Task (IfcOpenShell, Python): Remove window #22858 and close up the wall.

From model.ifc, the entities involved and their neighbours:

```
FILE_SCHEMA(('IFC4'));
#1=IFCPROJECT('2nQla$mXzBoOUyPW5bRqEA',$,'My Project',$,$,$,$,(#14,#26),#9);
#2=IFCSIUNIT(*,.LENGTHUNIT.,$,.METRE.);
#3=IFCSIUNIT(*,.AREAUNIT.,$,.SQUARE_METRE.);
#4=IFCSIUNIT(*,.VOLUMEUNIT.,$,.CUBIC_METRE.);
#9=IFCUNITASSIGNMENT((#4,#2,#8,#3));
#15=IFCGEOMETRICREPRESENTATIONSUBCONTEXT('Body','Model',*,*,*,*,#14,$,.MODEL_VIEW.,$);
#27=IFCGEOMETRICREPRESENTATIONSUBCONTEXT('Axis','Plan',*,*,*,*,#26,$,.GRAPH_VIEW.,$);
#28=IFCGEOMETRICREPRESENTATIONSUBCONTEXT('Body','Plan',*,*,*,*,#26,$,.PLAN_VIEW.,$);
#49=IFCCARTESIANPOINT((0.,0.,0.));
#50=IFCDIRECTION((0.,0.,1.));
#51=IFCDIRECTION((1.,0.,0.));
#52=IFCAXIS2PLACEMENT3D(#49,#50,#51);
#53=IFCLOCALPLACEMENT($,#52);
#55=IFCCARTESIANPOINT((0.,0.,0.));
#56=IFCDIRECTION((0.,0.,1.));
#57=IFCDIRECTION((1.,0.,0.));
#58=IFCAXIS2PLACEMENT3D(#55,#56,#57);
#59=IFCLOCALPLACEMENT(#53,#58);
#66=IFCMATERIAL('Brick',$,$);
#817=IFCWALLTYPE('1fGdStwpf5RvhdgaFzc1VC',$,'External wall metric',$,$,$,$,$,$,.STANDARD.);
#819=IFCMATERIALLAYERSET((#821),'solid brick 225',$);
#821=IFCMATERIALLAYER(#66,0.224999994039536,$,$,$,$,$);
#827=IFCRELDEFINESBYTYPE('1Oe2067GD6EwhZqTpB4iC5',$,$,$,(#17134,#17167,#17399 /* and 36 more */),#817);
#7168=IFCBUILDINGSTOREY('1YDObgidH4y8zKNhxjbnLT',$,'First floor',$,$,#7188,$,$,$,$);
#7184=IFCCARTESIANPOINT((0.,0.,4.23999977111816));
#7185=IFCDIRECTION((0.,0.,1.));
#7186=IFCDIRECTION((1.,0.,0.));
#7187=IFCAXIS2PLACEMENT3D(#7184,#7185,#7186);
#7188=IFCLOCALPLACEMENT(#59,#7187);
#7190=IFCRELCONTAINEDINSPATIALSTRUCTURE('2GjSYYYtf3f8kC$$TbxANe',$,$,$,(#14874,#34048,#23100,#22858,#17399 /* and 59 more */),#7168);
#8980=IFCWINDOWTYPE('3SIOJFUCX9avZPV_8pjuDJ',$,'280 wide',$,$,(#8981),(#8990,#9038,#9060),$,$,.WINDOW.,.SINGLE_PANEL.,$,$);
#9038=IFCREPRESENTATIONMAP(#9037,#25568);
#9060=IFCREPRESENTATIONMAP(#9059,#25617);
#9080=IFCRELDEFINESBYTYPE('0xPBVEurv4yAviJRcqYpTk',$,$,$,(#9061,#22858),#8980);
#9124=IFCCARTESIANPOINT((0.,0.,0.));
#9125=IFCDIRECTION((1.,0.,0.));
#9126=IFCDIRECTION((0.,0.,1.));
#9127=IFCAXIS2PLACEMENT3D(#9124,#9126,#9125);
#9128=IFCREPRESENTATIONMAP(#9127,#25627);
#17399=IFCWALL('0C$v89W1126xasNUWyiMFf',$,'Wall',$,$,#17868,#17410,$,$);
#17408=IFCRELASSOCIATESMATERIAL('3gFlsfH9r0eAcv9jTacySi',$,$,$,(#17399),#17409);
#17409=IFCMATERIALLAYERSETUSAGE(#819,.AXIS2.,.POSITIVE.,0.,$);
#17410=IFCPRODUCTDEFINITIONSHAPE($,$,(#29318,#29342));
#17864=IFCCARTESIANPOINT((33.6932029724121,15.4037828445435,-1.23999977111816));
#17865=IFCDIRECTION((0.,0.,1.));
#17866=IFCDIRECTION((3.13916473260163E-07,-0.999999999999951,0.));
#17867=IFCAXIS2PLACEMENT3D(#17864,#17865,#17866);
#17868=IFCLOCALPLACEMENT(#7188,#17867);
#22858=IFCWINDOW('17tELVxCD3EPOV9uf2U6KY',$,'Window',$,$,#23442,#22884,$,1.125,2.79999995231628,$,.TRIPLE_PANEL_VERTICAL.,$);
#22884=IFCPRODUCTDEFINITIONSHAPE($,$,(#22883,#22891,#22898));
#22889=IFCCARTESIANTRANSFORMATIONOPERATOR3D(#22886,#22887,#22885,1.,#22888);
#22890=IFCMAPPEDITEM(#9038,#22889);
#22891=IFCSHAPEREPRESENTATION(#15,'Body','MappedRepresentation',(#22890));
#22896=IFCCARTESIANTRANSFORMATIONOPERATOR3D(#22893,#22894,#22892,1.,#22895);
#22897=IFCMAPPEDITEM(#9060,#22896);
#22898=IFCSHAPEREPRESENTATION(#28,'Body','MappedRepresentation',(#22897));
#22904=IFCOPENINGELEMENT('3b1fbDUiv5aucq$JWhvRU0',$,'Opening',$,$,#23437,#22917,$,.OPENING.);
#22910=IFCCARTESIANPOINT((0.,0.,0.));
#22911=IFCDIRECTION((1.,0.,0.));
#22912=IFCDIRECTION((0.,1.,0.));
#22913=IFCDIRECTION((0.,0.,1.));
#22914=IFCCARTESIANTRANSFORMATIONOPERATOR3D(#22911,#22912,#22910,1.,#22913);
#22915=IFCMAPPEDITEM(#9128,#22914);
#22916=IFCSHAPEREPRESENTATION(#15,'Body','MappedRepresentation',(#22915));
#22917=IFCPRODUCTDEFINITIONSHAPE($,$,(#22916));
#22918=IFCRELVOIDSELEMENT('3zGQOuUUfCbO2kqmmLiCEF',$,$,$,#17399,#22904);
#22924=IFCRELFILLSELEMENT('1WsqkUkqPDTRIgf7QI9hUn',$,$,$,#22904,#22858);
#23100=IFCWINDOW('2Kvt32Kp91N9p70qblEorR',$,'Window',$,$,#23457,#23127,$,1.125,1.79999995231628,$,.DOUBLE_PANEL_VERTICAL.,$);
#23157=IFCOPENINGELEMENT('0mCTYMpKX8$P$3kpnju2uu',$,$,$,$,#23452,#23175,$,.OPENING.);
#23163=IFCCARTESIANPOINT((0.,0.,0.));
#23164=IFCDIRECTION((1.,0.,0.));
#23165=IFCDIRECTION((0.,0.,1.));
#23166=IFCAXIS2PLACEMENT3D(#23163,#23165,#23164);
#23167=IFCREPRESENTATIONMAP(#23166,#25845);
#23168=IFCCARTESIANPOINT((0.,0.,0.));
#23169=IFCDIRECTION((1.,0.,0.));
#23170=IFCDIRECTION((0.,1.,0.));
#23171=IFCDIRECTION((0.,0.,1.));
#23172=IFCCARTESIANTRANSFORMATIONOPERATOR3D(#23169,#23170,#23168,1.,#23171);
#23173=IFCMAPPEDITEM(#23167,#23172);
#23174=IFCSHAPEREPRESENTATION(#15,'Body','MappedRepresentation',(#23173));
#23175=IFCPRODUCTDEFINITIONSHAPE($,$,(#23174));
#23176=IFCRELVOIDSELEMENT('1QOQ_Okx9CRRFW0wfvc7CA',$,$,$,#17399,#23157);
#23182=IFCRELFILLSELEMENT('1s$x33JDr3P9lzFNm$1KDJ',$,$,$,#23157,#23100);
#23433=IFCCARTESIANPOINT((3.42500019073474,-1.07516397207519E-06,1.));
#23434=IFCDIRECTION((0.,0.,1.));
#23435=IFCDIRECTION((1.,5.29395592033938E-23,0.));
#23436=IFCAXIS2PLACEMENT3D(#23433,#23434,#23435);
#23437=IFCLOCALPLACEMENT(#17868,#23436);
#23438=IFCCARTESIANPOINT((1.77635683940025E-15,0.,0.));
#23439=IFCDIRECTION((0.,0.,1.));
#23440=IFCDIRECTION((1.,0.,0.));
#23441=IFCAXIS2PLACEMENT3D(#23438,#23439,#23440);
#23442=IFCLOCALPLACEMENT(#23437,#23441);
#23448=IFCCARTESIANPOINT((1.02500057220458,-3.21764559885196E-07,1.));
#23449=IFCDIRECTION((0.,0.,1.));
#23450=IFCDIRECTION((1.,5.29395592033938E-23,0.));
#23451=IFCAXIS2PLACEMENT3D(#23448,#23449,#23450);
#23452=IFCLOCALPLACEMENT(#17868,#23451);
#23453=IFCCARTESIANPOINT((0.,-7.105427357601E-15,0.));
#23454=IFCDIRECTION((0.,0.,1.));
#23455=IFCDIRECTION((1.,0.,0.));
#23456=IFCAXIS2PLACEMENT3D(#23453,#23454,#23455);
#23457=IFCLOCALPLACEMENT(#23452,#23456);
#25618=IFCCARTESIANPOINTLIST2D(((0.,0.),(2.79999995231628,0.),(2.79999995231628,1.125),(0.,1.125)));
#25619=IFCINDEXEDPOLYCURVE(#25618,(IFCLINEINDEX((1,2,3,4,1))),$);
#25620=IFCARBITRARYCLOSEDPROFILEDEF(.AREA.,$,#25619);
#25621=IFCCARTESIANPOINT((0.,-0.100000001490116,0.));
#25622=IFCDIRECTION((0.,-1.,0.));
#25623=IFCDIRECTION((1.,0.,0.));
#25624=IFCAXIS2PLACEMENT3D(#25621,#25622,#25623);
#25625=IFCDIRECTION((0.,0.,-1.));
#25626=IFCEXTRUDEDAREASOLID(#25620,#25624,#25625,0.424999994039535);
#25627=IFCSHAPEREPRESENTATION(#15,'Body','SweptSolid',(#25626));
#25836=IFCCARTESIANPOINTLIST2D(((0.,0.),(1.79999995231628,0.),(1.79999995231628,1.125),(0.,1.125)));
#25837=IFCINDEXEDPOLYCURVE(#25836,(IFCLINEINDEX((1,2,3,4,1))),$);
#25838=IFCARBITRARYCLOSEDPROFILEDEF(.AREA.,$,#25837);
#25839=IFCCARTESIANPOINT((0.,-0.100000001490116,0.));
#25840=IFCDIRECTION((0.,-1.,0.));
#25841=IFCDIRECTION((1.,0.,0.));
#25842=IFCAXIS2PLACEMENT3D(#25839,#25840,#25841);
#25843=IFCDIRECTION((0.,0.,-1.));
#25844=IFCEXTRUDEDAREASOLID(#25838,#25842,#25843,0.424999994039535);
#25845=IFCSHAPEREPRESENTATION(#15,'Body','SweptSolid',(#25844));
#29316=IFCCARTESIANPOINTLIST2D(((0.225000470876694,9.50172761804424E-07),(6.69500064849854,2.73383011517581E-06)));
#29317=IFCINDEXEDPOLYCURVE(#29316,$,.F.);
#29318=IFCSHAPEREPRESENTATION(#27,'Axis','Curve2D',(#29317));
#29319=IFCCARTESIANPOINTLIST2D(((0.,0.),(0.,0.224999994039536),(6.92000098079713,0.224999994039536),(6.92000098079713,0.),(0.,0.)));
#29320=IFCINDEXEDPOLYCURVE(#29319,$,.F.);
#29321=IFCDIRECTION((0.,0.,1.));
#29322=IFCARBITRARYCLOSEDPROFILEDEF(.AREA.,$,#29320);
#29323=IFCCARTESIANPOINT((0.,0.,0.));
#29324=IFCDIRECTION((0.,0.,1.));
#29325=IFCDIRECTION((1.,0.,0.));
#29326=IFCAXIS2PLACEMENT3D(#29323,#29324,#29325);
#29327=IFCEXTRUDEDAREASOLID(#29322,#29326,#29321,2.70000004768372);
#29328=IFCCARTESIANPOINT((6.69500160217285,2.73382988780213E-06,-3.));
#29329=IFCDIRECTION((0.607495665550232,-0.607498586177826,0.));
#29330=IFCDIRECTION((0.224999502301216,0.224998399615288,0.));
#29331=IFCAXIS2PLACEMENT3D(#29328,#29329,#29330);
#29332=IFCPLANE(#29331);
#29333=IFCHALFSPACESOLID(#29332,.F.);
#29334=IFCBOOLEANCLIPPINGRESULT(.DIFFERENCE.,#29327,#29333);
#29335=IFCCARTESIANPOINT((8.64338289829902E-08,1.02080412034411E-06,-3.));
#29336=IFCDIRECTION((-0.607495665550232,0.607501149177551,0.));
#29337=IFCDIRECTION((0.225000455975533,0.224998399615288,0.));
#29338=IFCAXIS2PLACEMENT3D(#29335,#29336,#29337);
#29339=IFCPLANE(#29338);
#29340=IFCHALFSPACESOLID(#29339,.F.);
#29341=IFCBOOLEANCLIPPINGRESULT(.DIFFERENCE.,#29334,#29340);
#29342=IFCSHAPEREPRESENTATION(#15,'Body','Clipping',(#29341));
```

```python
import ifcopenshell
import ifcopenshell.api.feature
import ifcopenshell.api.root
import ifcopenshell.geom
import ifcopenshell.util.shape

model = ifcopenshell.open("model.ifc")
settings = ifcopenshell.geom.settings()


def volume(element):
    """Net volume in cubic metres, openings subtracted."""
    shape = ifcopenshell.geom.create_shape(settings, element)
    return ifcopenshell.util.shape.get_volume(shape.geometry)


window = model.by_id(22858)
opening = window.FillsVoids[0].RelatingOpeningElement
wall = opening.VoidsElements[0].RelatingBuildingElement
before = volume(wall)

ifcopenshell.api.root.remove_product(model, product=window)
ifcopenshell.api.feature.remove_feature(model, feature=opening)

after = volume(wall)

print(f"wall volume {before:.3f} -> {after:.3f} m3")

model.write("model-out.ifc")
```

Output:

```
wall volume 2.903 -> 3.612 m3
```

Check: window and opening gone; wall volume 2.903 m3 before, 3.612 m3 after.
